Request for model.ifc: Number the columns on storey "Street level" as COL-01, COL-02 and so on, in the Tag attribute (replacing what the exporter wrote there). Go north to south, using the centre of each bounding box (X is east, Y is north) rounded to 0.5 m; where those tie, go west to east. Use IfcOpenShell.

First a look at what the model holds.

```python
import ifcopenshell
import ifcopenshell.util.element
import ifcopenshell.util.placement

model = ifcopenshell.open("model.ifc")
print(model.schema)
storey = next(s for s in model.by_type("IfcBuildingStorey") if s.Name == "Street level")
columns = [e for e in ifcopenshell.util.element.get_decomposition(storey) if e.is_a("IfcColumn")]
for e in sorted(columns, key=lambda e: e.id()):
    origin = ifcopenshell.util.placement.get_local_placement(e.ObjectPlacement)[:3, 3]
    print(e.id(), e.Tag, e.Name, origin.round(2) + 0.0, sep=" | ")
```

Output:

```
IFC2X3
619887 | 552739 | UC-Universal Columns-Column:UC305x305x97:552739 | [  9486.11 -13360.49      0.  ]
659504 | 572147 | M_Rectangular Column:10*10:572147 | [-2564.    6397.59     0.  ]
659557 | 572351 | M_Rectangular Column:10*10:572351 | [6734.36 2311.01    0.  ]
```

```python
import ifcopenshell
import ifcopenshell.geom
import ifcopenshell.util.element
import ifcopenshell.util.shape

model = ifcopenshell.open("model.ifc")
settings = ifcopenshell.geom.settings()
settings.set("use-world-coords", True)


def centre(element):
    shape = ifcopenshell.geom.create_shape(settings, element)
    return ifcopenshell.util.shape.get_bbox_centroid(shape.geometry)


storey = next(s for s in model.by_type("IfcBuildingStorey") if s.Name == "Street level")
columns = [e for e in ifcopenshell.util.element.get_decomposition(storey) if e.is_a("IfcColumn")]

# Insertion points can sit at a corner or the storey origin, so sort by the geometry (in metres).
centres = {e: centre(e) for e in columns}
columns.sort(key=lambda e: (-round(centres[e][1] / 0.5), centres[e][0]))

for i, e in enumerate(columns, start=1):
    number = f"COL-{i:02d}"
    e.Tag = number
    print(e.id(), number)

model.write("model_edited.ifc")
```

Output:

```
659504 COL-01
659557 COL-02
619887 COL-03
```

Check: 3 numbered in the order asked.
